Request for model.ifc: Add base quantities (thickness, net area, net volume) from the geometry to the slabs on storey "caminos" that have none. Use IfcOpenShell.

First a look at what the model holds.

```python
import ifcopenshell
import ifcopenshell.util.element
import ifcopenshell.util.unit

model = ifcopenshell.open("model.ifc")
print(model.schema)
for unit_type in ("LENGTHUNIT", "AREAUNIT", "VOLUMEUNIT"):
    print(unit_type, ifcopenshell.util.unit.calculate_unit_scale(model, unit_type))
storey = next(s for s in model.by_type("IfcBuildingStorey") if s.Name == "caminos")
slabs = [e for e in ifcopenshell.util.element.get_decomposition(storey) if e.is_a("IfcSlab")]
for e in sorted(slabs, key=lambda e: e.id()):
    print(e.id(), e.is_a(), e.Name, list(ifcopenshell.util.element.get_psets(e, qtos_only=True)), sep=" | ")
```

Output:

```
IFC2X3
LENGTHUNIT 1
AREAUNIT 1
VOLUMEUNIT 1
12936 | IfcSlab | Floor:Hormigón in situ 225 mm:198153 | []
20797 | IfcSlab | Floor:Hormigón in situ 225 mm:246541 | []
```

```python
import ifcopenshell
import ifcopenshell.api.pset
import ifcopenshell.geom
import ifcopenshell.util.element
import ifcopenshell.util.shape
import ifcopenshell.util.unit

model = ifcopenshell.open("model.ifc")
unit_scale = ifcopenshell.util.unit.calculate_unit_scale(model)
area_scale = ifcopenshell.util.unit.calculate_unit_scale(model, "AREAUNIT")
volume_scale = ifcopenshell.util.unit.calculate_unit_scale(model, "VOLUMEUNIT")
settings = ifcopenshell.geom.settings()

storey = next(s for s in model.by_type("IfcBuildingStorey") if s.Name == "caminos")
slabs = [e for e in ifcopenshell.util.element.get_decomposition(storey) if e.is_a("IfcSlab")]

for e in sorted(slabs, key=lambda e: e.id()):
    if ifcopenshell.util.element.get_psets(e, qtos_only=True, should_inherit=False):
        continue
    # Geometry comes back in metres, in the element's own axes.
    shape = ifcopenshell.geom.create_shape(settings, e)
    values = {
        "Width": ifcopenshell.util.shape.get_z(shape.geometry) / unit_scale,
        "NetArea": ifcopenshell.util.shape.get_footprint_area(shape.geometry) / area_scale,
        "NetVolume": ifcopenshell.util.shape.get_volume(shape.geometry) / volume_scale,
    }
    qto = ifcopenshell.api.pset.add_qto(model, product=e, name="BaseQuantities")
    ifcopenshell.api.pset.edit_qto(model, qto=qto, properties=values)
    print(e.id(), {k: round(v, 3) for k, v in values.items()})

model.write("model_updated.ifc")
```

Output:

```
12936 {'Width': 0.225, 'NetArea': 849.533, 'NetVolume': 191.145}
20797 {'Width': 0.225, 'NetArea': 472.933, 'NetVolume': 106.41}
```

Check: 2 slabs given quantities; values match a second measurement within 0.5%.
